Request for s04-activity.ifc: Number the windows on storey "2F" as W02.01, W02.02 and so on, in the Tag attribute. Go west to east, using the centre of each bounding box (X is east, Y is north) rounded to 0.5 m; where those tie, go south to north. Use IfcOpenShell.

First a look at what the model holds.

```python
import ifcopenshell
import ifcopenshell.util.element
import ifcopenshell.util.placement

model = ifcopenshell.open("s04-activity.ifc")
print(model.schema)
storey = next(s for s in model.by_type("IfcBuildingStorey") if s.Name == "2F")
windows = [e for e in ifcopenshell.util.element.get_decomposition(storey) if e.is_a("IfcWindow")]
for e in sorted(windows, key=lambda e: e.id()):
    origin = ifcopenshell.util.placement.get_local_placement(e.ObjectPlacement)[:3, 3]
    print(e.id(), e.Tag, e.Name, origin.round(2) + 0.0, sep=" | ")
```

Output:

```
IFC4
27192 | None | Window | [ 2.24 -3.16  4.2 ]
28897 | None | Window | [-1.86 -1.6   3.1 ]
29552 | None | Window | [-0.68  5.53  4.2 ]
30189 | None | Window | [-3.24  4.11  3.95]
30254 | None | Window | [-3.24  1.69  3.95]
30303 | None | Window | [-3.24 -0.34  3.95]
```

```python
import ifcopenshell
import ifcopenshell.geom
import ifcopenshell.util.element
import ifcopenshell.util.shape

model = ifcopenshell.open("s04-activity.ifc")
settings = ifcopenshell.geom.settings()
settings.set("use-world-coords", True)


def centre(element):
    shape = ifcopenshell.geom.create_shape(settings, element)
    return ifcopenshell.util.shape.get_bbox_centroid(shape.geometry)


storey = next(s for s in model.by_type("IfcBuildingStorey") if s.Name == "2F")
windows = [e for e in ifcopenshell.util.element.get_decomposition(storey) if e.is_a("IfcWindow")]

# Insertion points can sit at a corner or the storey origin, so sort by the geometry (in metres).
centres = {e: centre(e) for e in windows}
windows.sort(key=lambda e: (round(centres[e][0] / 0.5), centres[e][1]))

for i, e in enumerate(windows, start=1):
    number = f"W02.{i:02d}"
    e.Tag = number
    print(e.id(), number)

model.write("s04-activity_v2.ifc")
```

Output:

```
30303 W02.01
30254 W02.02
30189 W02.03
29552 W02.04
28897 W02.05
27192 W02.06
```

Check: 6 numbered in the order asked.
